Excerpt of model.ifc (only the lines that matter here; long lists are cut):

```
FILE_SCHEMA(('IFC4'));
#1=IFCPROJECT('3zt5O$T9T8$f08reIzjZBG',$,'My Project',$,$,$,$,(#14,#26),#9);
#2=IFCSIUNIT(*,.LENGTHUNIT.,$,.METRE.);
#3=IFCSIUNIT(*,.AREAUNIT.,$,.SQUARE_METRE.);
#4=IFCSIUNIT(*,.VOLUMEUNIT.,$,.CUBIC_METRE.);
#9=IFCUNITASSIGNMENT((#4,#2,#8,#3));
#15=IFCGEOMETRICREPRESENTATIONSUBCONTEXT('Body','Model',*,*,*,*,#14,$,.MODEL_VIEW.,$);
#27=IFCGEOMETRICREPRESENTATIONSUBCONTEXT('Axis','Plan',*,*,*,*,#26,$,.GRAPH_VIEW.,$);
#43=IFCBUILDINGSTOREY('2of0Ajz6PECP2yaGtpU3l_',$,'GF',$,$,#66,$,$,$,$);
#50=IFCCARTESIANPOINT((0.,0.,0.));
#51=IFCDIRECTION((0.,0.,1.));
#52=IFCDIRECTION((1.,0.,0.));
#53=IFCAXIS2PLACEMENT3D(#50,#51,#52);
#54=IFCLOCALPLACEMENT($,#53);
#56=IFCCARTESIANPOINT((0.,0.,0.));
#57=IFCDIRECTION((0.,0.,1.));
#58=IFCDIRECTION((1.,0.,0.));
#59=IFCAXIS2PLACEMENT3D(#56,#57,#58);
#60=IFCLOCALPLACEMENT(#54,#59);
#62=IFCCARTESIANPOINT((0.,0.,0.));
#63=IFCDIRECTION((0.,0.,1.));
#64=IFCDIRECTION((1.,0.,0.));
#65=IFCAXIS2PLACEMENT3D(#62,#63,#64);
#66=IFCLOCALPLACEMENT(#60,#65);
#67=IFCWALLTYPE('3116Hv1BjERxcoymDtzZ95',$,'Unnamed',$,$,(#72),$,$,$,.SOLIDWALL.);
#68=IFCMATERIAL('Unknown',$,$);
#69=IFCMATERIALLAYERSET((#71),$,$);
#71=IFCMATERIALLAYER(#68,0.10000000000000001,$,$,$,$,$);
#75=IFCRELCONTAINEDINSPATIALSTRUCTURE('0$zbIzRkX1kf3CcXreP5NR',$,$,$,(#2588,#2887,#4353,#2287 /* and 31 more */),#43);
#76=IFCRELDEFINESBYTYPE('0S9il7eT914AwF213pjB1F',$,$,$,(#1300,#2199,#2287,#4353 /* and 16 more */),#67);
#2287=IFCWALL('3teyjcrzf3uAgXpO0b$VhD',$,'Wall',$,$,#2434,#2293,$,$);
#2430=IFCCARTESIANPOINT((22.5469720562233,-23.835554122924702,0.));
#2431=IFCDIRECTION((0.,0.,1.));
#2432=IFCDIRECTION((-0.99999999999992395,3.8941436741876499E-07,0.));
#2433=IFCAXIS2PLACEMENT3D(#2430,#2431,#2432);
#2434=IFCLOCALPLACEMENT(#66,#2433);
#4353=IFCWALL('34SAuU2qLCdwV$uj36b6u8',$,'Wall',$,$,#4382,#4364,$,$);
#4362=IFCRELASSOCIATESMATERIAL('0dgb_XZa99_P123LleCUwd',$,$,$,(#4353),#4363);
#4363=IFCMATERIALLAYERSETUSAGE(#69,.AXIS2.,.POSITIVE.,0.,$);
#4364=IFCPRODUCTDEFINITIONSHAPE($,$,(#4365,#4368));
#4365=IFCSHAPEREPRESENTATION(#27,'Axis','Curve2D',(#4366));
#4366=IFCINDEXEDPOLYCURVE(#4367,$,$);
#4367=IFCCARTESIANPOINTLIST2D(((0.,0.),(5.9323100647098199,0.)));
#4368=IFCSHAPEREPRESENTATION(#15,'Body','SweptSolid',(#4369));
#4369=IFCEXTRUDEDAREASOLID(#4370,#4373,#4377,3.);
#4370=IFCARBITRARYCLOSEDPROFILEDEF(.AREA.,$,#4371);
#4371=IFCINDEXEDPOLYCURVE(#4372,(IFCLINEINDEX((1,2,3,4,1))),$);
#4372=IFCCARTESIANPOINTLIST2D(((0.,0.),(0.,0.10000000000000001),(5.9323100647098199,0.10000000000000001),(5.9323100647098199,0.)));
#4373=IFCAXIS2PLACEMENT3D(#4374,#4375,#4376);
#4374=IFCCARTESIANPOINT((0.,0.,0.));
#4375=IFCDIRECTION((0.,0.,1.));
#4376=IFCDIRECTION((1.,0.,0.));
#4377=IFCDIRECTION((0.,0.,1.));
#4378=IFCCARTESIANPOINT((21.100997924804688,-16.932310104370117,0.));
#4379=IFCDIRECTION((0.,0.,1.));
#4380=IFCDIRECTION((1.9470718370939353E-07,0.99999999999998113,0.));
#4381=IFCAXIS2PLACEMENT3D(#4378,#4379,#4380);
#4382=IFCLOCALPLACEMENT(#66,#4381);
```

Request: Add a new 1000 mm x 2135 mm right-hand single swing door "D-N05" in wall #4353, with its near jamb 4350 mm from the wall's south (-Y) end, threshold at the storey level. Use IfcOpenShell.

```python
import numpy as np
import ifcopenshell
import ifcopenshell.api.feature
import ifcopenshell.api.geometry
import ifcopenshell.api.root
import ifcopenshell.api.spatial
import ifcopenshell.geom
import ifcopenshell.util.element
import ifcopenshell.util.placement
import ifcopenshell.util.representation
import ifcopenshell.util.shape
import ifcopenshell.util.unit

model = ifcopenshell.open("model.ifc")
unit_scale = ifcopenshell.util.unit.calculate_unit_scale(model)
settings = ifcopenshell.geom.settings()


def volume(element):
    """Net volume in cubic metres, openings subtracted."""
    shape = ifcopenshell.geom.create_shape(settings, element)
    return ifcopenshell.util.shape.get_volume(shape.geometry)


wall = model.by_id(4353)
storey = ifcopenshell.util.element.get_container(wall, ifc_class="IfcBuildingStorey")
context = ifcopenshell.util.representation.get_context(model, "Model", "Body", "MODEL_VIEW")
before = volume(wall)

width, height, from_end, sill = 1, 2.135, 4.35, 0.0  # metres

# The wall runs along its own X axis, and the end named is its -X end.
wall_shape = ifcopenshell.geom.create_shape(settings, wall)
x, y, z = ifcopenshell.util.shape.get_vertices(wall_shape.geometry).T
start = x.min() + from_end
face, thickness = float(y.min()), float(y.max() - y.min())
wall_matrix = ifcopenshell.util.placement.get_local_placement(wall.ObjectPlacement)
level = ifcopenshell.util.placement.get_local_placement(storey.ObjectPlacement)[2, 3]


def in_wall(x, y):
    """Placement at x, y metres in the wall's axes, at sill height."""
    matrix = wall_matrix.copy()
    matrix[:, 3] = wall_matrix @ np.array([x / unit_scale, y / unit_scale, 0.0, 1.0])
    matrix[2, 3] = level + sill / unit_scale
    return matrix


# Opening: a box that overshoots both wall faces by 50 mm.
opening = ifcopenshell.api.root.create_entity(model, ifc_class="IfcOpeningElement", predefined_type="OPENING")
box = ifcopenshell.api.geometry.add_wall_representation(
    model, context=context, length=width, height=height, thickness=thickness + 0.1
)
ifcopenshell.api.geometry.assign_representation(model, product=opening, representation=box)
ifcopenshell.api.geometry.edit_object_placement(model, product=opening, matrix=in_wall(start, face - 0.05), is_si=False)
ifcopenshell.api.feature.add_feature(model, feature=opening, element=wall)

door = ifcopenshell.api.root.create_entity(model, ifc_class="IfcDoor", name="D-N05", predefined_type="DOOR")
door.OverallWidth, door.OverallHeight = width / unit_scale, height / unit_scale
door.OperationType = "SINGLE_SWING_RIGHT"
body = ifcopenshell.api.geometry.add_door_representation(
    model,
    context=context,
    overall_width=door.OverallWidth,
    overall_height=door.OverallHeight,
    operation_type="SINGLE_SWING_RIGHT",
    lining_properties={"LiningDepth": thickness / unit_scale, "ThresholdDepth": thickness / unit_scale},
)
ifcopenshell.api.geometry.assign_representation(model, product=door, representation=body)
ifcopenshell.api.spatial.assign_container(model, products=[door], relating_structure=storey)
ifcopenshell.api.feature.add_filling(model, opening=opening, element=door)

# The lining spans the wall, so the door starts at the wall face.
ifcopenshell.api.geometry.edit_object_placement(model, product=door, matrix=in_wall(start, face), is_si=False)

after = volume(wall)

print(f"wall volume {before:.3f} -> {after:.3f} m3")

model.write("model_rev.ifc")
```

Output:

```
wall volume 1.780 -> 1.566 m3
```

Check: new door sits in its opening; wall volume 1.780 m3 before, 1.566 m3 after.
